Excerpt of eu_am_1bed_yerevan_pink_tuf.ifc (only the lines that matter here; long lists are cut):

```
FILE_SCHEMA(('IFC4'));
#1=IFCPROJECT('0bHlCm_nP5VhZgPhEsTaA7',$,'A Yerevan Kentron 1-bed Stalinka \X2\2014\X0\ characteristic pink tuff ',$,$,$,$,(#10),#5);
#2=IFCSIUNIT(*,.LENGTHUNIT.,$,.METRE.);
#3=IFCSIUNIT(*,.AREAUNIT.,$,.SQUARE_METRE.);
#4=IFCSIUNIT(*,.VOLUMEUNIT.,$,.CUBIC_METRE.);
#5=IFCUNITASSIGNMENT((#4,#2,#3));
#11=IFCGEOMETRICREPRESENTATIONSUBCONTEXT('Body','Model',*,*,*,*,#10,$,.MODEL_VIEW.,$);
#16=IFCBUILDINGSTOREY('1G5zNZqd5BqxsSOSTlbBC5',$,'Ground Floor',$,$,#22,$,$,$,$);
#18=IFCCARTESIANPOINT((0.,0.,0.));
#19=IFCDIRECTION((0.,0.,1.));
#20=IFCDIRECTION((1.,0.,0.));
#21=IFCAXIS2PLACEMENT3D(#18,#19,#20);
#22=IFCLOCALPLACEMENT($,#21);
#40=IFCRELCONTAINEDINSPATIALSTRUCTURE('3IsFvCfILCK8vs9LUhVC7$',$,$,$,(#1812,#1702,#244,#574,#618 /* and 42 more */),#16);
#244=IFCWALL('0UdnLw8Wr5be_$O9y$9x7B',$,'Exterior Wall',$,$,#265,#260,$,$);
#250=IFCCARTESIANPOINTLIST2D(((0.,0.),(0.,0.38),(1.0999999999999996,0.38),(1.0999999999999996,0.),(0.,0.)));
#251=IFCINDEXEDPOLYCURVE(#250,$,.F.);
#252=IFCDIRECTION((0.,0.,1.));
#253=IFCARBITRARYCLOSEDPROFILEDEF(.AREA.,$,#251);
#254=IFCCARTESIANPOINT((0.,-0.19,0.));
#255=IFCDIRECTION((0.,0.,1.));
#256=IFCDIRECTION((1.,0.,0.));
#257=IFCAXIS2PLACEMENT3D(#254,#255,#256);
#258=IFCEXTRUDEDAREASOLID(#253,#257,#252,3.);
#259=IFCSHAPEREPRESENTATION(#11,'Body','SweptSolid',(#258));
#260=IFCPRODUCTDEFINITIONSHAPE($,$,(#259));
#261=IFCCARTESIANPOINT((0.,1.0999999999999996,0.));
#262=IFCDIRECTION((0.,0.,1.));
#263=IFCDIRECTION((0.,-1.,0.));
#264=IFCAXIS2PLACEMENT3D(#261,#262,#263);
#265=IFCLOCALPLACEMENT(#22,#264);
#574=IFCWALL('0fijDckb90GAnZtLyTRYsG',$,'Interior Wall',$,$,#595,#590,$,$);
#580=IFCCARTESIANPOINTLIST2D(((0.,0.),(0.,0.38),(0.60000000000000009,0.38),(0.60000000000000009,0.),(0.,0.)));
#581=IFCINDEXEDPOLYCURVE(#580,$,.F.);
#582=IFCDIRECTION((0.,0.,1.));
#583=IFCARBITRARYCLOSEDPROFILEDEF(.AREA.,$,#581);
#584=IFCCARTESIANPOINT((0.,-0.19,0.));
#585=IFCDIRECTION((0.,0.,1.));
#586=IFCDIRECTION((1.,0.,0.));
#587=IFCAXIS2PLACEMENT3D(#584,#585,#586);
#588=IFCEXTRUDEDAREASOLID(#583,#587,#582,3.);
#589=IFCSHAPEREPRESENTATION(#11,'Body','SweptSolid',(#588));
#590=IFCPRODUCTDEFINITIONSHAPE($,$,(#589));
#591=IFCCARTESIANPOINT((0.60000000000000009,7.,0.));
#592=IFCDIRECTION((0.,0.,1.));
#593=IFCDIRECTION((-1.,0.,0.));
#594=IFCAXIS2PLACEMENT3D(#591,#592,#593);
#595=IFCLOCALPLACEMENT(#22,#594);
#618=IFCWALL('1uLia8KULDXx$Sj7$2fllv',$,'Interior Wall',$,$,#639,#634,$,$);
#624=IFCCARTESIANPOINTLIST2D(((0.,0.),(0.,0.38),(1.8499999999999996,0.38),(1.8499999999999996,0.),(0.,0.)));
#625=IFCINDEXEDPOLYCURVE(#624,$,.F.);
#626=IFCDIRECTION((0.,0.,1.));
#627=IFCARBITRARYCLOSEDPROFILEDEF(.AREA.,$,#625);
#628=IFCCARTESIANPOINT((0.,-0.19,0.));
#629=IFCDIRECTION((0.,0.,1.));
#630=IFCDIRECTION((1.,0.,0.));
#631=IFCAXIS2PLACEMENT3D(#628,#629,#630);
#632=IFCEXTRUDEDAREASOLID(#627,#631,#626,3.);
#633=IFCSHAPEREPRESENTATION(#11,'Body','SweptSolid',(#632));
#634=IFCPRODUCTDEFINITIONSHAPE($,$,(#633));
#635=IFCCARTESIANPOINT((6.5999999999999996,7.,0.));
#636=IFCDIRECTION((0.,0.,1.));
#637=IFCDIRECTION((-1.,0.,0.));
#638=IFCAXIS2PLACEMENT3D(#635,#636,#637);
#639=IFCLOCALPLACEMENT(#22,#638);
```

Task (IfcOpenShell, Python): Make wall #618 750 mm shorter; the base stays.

```python
import ifcopenshell
import ifcopenshell.geom
import ifcopenshell.util.representation
import ifcopenshell.util.shape
import ifcopenshell.util.unit

model = ifcopenshell.open("eu_am_1bed_yerevan_pink_tuf.ifc")
unit_scale = ifcopenshell.util.unit.calculate_unit_scale(model)
settings = ifcopenshell.geom.settings()


def volume(element):
    """Net volume in cubic metres, openings subtracted."""
    shape = ifcopenshell.geom.create_shape(settings, element)
    return ifcopenshell.util.shape.get_volume(shape.geometry)


wall = model.by_guid("1uLia8KULDXx$Sj7$2fllv")
before = volume(wall)

body = ifcopenshell.util.representation.get_representation(wall, "Model", "Body")
solid = body.Items[0]
old_height = solid.Depth
solid.Depth -= 0.75 / unit_scale
after = volume(wall)

print(f"height {old_height:g} -> {solid.Depth:g}, volume {before:.3f} -> {after:.3f} m3")

model.write("eu_am_1bed_yerevan_pink_tuf_edited.ifc")
```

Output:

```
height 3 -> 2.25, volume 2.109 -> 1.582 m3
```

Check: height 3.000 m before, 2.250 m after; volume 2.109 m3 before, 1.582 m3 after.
